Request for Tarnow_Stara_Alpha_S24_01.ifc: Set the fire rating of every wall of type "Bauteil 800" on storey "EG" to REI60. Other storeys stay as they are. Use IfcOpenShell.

First a look at what the model holds.

```python
import ifcopenshell
import ifcopenshell.util.element

model = ifcopenshell.open("Tarnow_Stara_Alpha_S24_01.ifc")
print(model.schema)
storey = next(s for s in model.by_type("IfcBuildingStorey") if s.Name == "EG")
walls = [e for e in ifcopenshell.util.element.get_decomposition(storey) if e.is_a("IfcWall")]
seen = {}
for e in walls:
    element_type = ifcopenshell.util.element.get_type(e)
    key = (element_type.Name if element_type != e and element_type else None, ifcopenshell.util.element.get_pset(e, "Pset_WallCommon", "FireRating"))
    seen[key] = seen.get(key, 0) + 1
for (name, value), count in sorted(seen.items(), key=str):
    print(count, "x", name, "|", value)
```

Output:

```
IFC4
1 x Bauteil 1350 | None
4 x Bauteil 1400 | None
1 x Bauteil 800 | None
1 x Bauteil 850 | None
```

```python
import ifcopenshell
import ifcopenshell.api.pset
import ifcopenshell.util.element

model = ifcopenshell.open("Tarnow_Stara_Alpha_S24_01.ifc")

storey = next(s for s in model.by_type("IfcBuildingStorey") if s.Name == "EG")
walls = [e for e in ifcopenshell.util.element.get_decomposition(storey) if e.is_a("IfcWall")]

count = 0
for e in walls:
    element_type = ifcopenshell.util.element.get_type(e)
    if element_type in (None, e) or element_type.Name != "Bauteil 800":
        continue
    # add_pset returns the element's existing set when there is one.
    pset = ifcopenshell.api.pset.add_pset(model, product=e, name="Pset_WallCommon")
    ifcopenshell.api.pset.edit_pset(model, pset=pset, properties={"FireRating": "REI60"})
    count += 1

print(count, "walls updated")

model.write("Tarnow_Stara_Alpha_S24_01_edited.ifc")
```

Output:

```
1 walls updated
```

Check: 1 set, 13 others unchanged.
